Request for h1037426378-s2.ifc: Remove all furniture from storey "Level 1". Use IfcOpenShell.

First a look at what the model holds.

```python
import ifcopenshell
import ifcopenshell.util.element

model = ifcopenshell.open("h1037426378-s2.ifc")
print(model.schema)
storey = next(s for s in model.by_type("IfcBuildingStorey") if s.Name == "Level 1")
furniture = [e for e in ifcopenshell.util.element.get_decomposition(storey) if e.is_a("IfcFurnishingElement")]
seen = {}
for e in furniture:
    element_type = ifcopenshell.util.element.get_type(e)
    name = element_type.Name if element_type not in (None, e) else None
    seen[name] = seen.get(name, 0) + 1
for name, count in sorted(seen.items(), key=str):
    print(count, "x", name)
```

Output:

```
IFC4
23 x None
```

```python
import ifcopenshell
import ifcopenshell.api.root
import ifcopenshell.util.element

model = ifcopenshell.open("h1037426378-s2.ifc")

storey = next(s for s in model.by_type("IfcBuildingStorey") if s.Name == "Level 1")
furniture = [e for e in ifcopenshell.util.element.get_decomposition(storey) if e.is_a("IfcFurnishingElement")]

for e in furniture:
    ifcopenshell.api.root.remove_product(model, product=e)
print(len(furniture), "removed")

model.write("h1037426378-s2_edited.ifc")
```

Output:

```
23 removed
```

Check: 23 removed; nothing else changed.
